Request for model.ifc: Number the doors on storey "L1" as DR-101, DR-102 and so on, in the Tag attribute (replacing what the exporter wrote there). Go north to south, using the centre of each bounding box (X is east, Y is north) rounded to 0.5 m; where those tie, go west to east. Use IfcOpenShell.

First a look at what the model holds.

```python
import ifcopenshell
import ifcopenshell.util.element
import ifcopenshell.util.placement

model = ifcopenshell.open("model.ifc")
print(model.schema)
storey = next(s for s in model.by_type("IfcBuildingStorey") if s.Name == "L1")
doors = [e for e in ifcopenshell.util.element.get_decomposition(storey) if e.is_a("IfcDoor")]
for e in sorted(doors, key=lambda e: e.id()):
    origin = ifcopenshell.util.placement.get_local_placement(e.ObjectPlacement)[:3, 3]
    print(e.id(), e.Tag, e.Name, origin.round(2) + 0.0, sep=" | ")
```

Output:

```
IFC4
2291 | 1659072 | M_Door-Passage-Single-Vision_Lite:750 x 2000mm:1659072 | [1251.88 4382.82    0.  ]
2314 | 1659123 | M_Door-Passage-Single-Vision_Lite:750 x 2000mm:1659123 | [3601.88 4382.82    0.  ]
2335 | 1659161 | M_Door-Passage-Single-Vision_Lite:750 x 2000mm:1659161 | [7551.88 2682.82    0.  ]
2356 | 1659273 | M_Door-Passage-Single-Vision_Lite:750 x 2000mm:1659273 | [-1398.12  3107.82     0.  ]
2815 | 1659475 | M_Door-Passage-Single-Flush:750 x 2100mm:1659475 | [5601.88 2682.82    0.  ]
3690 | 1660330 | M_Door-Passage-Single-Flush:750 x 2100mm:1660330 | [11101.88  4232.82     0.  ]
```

```python
import ifcopenshell
import ifcopenshell.geom
import ifcopenshell.util.element
import ifcopenshell.util.shape

model = ifcopenshell.open("model.ifc")
settings = ifcopenshell.geom.settings()
settings.set("use-world-coords", True)


def centre(element):
    shape = ifcopenshell.geom.create_shape(settings, element)
    return ifcopenshell.util.shape.get_bbox_centroid(shape.geometry)


storey = next(s for s in model.by_type("IfcBuildingStorey") if s.Name == "L1")
doors = [e for e in ifcopenshell.util.element.get_decomposition(storey) if e.is_a("IfcDoor")]

# Insertion points can sit at a corner or the storey origin, so sort by the geometry (in metres).
centres = {e: centre(e) for e in doors}
doors.sort(key=lambda e: (-round(centres[e][1] / 0.5), centres[e][0]))

for i, e in enumerate(doors, start=1):
    number = f"DR-1{i:02d}"
    e.Tag = number
    print(e.id(), number)

model.write("model_edited.ifc")
```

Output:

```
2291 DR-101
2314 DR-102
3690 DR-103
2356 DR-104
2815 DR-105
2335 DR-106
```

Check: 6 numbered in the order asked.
